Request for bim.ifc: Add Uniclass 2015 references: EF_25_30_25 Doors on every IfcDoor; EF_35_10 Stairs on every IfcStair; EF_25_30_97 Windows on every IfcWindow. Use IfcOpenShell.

First a look at what the model holds.

```python
import ifcopenshell

model = ifcopenshell.open("bim.ifc")
print(model.schema)
print("classifications:", [c.Name for c in model.by_type("IfcClassification")])
for ifc_class in ("IfcDoor", "IfcRoof", "IfcStair", "IfcWall", "IfcWindow"):
    print(ifc_class, len(model.by_type(ifc_class)))
```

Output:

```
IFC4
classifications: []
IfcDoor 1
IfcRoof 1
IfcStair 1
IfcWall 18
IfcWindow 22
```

```python
import ifcopenshell
import ifcopenshell.api.classification

model = ifcopenshell.open("bim.ifc")

system = ifcopenshell.api.classification.add_classification(model, classification="Uniclass 2015")

codes = {
    "IfcDoor": ("EF_25_30_25", "Doors"),
    "IfcStair": ("EF_35_10", "Stairs"),
    "IfcWindow": ("EF_25_30_97", "Windows"),
}
for ifc_class, (code, name) in codes.items():
    products = model.by_type(ifc_class)
    ifcopenshell.api.classification.add_reference(
        model, products=products, classification=system, identification=code, name=name
    )
    print(code, len(products))

model.write("bim_rev.ifc")
```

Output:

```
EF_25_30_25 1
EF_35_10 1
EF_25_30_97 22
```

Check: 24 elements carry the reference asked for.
